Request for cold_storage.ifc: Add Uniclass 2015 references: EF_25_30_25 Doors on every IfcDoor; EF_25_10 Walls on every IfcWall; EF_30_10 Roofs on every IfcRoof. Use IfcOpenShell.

First a look at what the model holds.

```python
import ifcopenshell

model = ifcopenshell.open("cold_storage.ifc")
print(model.schema)
print("classifications:", [c.Name for c in model.by_type("IfcClassification")])
for ifc_class in ("IfcDoor", "IfcRoof", "IfcStair", "IfcWall", "IfcWindow"):
    print(ifc_class, len(model.by_type(ifc_class)))
```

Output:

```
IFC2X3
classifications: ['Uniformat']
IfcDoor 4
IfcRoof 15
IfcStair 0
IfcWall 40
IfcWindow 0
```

```python
import ifcopenshell
import ifcopenshell.api.classification

model = ifcopenshell.open("cold_storage.ifc")

# IFC2X3 requires Source and Edition and has no link from the project to the system.
system = model.create_entity("IfcClassification", Source="NBS", Edition="2015", Name="Uniclass 2015")

codes = {
    "IfcDoor": ("EF_25_30_25", "Doors"),
    "IfcWall": ("EF_25_10", "Walls"),
    "IfcRoof": ("EF_30_10", "Roofs"),
}
for ifc_class, (code, name) in codes.items():
    products = model.by_type(ifc_class)
    ifcopenshell.api.classification.add_reference(
        model, products=products, classification=system, identification=code, name=name
    )
    print(code, len(products))

model.write("cold_storage_rev.ifc")
```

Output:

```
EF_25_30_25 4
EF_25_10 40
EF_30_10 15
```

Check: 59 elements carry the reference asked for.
